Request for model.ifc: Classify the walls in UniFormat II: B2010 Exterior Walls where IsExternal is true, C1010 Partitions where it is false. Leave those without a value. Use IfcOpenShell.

First a look at what the model holds.

```python
import ifcopenshell
import ifcopenshell.util.element

model = ifcopenshell.open("model.ifc")
print(model.schema)
print("classifications:", [c.Name for c in model.by_type("IfcClassification")])
values = [ifcopenshell.util.element.get_pset(e, "Pset_WallCommon", "IsExternal") for e in model.by_type("IfcWall")]
for value in (True, False, None):
    print("IsExternal", value, values.count(value))
```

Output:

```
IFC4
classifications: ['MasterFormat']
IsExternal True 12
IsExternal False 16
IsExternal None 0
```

```python
import ifcopenshell
import ifcopenshell.api.classification
import ifcopenshell.util.element

model = ifcopenshell.open("model.ifc")

system = ifcopenshell.api.classification.add_classification(model, classification="UniFormat II")

walls = model.by_type("IfcWall")
external = {e: ifcopenshell.util.element.get_pset(e, "Pset_WallCommon", "IsExternal") for e in walls}
for flag, code, name in ((True, "B2010", "Exterior Walls"), (False, "C1010", "Partitions")):
    products = [e for e in walls if external[e] is flag]
    ifcopenshell.api.classification.add_reference(
        model, products=products, classification=system, identification=code, name=name
    )
    print(code, len(products))

model.write("model_edited.ifc")
```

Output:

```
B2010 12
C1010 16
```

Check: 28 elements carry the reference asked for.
